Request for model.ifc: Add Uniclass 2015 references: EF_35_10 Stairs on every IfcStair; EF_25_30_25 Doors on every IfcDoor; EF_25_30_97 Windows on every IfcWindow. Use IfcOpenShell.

First a look at what the model holds.

```python
import ifcopenshell

model = ifcopenshell.open("model.ifc")
print(model.schema)
print("classifications:", [c.Name for c in model.by_type("IfcClassification")])
for ifc_class in ("IfcDoor", "IfcRoof", "IfcStair", "IfcWall", "IfcWindow"):
    print(ifc_class, len(model.by_type(ifc_class)))
```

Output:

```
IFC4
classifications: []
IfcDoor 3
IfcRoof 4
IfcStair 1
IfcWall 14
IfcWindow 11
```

```python
import ifcopenshell
import ifcopenshell.api.classification

model = ifcopenshell.open("model.ifc")

system = ifcopenshell.api.classification.add_classification(model, classification="Uniclass 2015")

codes = {
    "IfcStair": ("EF_35_10", "Stairs"),
    "IfcDoor": ("EF_25_30_25", "Doors"),
    "IfcWindow": ("EF_25_30_97", "Windows"),
}
for ifc_class, (code, name) in codes.items():
    products = model.by_type(ifc_class)
    ifcopenshell.api.classification.add_reference(
        model, products=products, classification=system, identification=code, name=name
    )
    print(code, len(products))

model.write("model_updated.ifc")
```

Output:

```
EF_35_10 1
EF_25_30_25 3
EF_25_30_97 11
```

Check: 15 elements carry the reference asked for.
